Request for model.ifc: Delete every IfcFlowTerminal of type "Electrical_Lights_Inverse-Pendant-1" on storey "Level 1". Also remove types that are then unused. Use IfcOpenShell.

First a look at what the model holds.

```python
import ifcopenshell
import ifcopenshell.util.element

model = ifcopenshell.open("model.ifc")
print(model.schema)
storey = next(s for s in model.by_type("IfcBuildingStorey") if s.Name == "Level 1")
terminals = [e for e in ifcopenshell.util.element.get_decomposition(storey) if e.is_a("IfcFlowTerminal")]
seen = {}
for e in terminals:
    element_type = ifcopenshell.util.element.get_type(e)
    name = element_type.Name if element_type not in (None, e) else None
    seen[name] = seen.get(name, 0) + 1
for name, count in sorted(seen.items(), key=str):
    print(count, "x", name)
```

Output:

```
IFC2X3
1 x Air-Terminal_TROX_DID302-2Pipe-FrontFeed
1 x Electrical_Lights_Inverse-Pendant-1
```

```python
import ifcopenshell
import ifcopenshell.api.root
import ifcopenshell.util.element

model = ifcopenshell.open("model.ifc")

storey = next(s for s in model.by_type("IfcBuildingStorey") if s.Name == "Level 1")
terminals = [e for e in ifcopenshell.util.element.get_decomposition(storey) if e.is_a("IfcFlowTerminal")]
targets = [e for e in terminals if (t := ifcopenshell.util.element.get_type(e)) not in (None, e) and t.Name == "Electrical_Lights_Inverse-Pendant-1"]
types = {ifcopenshell.util.element.get_type(e) for e in targets} - {None, *targets}

for e in targets:
    ifcopenshell.api.root.remove_product(model, product=e)
print(len(targets), "removed")

unused = [t for t in types if not ifcopenshell.util.element.get_types(t)]
for t in unused:
    ifcopenshell.api.root.remove_product(model, product=t)
print(len(unused), "unused types removed")

model.write("model_rev.ifc")
```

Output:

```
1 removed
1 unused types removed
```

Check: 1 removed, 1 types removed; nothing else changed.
